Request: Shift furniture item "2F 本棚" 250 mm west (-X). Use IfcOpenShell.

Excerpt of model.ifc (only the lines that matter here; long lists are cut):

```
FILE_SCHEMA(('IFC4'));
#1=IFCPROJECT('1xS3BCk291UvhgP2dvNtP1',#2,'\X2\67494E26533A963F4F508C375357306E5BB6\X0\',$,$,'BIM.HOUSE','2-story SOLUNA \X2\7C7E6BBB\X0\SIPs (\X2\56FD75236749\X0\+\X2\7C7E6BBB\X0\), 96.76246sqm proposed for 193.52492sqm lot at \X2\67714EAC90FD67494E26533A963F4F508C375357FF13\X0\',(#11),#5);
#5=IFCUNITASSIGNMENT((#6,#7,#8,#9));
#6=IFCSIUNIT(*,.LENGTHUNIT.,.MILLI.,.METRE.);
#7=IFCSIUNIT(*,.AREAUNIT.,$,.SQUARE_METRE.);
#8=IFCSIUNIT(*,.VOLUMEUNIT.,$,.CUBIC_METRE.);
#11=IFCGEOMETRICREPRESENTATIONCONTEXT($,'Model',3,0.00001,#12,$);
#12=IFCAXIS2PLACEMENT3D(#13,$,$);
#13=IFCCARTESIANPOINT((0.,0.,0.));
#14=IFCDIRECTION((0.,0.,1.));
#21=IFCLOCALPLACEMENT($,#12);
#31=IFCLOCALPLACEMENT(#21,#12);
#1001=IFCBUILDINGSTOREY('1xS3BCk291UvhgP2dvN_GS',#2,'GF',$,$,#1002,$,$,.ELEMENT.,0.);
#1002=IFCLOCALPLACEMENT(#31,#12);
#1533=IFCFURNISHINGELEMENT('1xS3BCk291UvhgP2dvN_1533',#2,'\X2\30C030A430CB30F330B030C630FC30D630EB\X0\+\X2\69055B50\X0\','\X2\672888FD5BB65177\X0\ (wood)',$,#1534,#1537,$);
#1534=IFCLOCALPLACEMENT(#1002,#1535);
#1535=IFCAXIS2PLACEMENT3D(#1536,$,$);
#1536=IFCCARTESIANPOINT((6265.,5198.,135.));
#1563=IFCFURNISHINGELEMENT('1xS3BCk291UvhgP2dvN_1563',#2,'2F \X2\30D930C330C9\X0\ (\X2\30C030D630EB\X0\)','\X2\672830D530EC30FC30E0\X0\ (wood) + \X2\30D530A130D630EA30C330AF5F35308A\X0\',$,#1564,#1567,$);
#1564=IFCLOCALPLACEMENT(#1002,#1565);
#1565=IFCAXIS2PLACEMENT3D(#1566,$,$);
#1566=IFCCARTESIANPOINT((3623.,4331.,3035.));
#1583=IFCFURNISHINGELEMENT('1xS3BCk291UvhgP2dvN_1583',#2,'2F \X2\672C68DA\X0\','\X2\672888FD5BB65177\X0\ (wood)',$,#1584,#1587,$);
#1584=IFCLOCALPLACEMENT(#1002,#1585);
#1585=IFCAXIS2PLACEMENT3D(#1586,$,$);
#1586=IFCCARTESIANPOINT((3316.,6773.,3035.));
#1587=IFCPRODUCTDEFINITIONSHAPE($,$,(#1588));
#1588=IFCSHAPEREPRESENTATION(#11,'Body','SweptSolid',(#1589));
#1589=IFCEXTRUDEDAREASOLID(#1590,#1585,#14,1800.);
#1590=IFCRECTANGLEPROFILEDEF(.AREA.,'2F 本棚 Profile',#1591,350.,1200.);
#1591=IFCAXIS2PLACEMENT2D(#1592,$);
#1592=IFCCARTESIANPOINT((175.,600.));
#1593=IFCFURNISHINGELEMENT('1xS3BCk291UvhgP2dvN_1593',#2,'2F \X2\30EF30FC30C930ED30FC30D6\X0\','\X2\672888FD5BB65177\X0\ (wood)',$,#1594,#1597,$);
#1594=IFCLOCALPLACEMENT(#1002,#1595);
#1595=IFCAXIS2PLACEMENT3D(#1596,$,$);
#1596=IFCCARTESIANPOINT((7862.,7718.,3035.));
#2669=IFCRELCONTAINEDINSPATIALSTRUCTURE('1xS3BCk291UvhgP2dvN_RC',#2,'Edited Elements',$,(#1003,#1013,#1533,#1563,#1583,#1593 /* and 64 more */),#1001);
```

```python
import ifcopenshell
import ifcopenshell.api.geometry
import ifcopenshell.util.placement

model = ifcopenshell.open("model.ifc")

item = model.by_guid("1xS3BCk291UvhgP2dvN_1583")
matrix = ifcopenshell.util.placement.get_local_placement(item.ObjectPlacement)
matrix[0, 3] -= 250.0
ifcopenshell.api.geometry.edit_object_placement(model, product=item, matrix=matrix, is_si=False)

print(ifcopenshell.util.placement.get_local_placement(item.ObjectPlacement).round(3) + 0.0)

model.write("model_v2.ifc")
```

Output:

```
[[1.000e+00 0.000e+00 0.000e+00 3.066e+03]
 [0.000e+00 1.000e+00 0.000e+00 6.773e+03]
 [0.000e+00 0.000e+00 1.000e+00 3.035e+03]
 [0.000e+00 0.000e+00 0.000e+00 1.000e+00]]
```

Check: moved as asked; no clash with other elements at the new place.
